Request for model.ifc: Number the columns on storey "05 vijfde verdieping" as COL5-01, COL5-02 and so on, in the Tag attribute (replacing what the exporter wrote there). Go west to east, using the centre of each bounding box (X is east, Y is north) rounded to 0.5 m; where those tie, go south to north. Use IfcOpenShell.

First a look at what the model holds.

```python
import ifcopenshell
import ifcopenshell.util.element
import ifcopenshell.util.placement

model = ifcopenshell.open("model.ifc")
print(model.schema)
storey = next(s for s in model.by_type("IfcBuildingStorey") if s.Name == "05 vijfde verdieping")
columns = [e for e in ifcopenshell.util.element.get_decomposition(storey) if e.is_a("IfcColumn")]
for e in sorted(columns, key=lambda e: e.id()):
    origin = ifcopenshell.util.placement.get_local_placement(e.ObjectPlacement)[:3, 3]
    print(e.id(), e.Tag, e.Name, origin.round(2) + 0.0, sep=" | ")
```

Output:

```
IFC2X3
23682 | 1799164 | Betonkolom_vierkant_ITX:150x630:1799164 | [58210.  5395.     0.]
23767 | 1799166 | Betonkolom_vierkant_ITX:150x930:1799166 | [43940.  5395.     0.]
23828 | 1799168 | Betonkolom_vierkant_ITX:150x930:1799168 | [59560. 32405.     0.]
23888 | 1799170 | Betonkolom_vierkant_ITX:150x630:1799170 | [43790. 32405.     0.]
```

```python
import ifcopenshell
import ifcopenshell.geom
import ifcopenshell.util.element
import ifcopenshell.util.shape

model = ifcopenshell.open("model.ifc")
settings = ifcopenshell.geom.settings()
settings.set("use-world-coords", True)


def centre(element):
    shape = ifcopenshell.geom.create_shape(settings, element)
    return ifcopenshell.util.shape.get_bbox_centroid(shape.geometry)


storey = next(s for s in model.by_type("IfcBuildingStorey") if s.Name == "05 vijfde verdieping")
columns = [e for e in ifcopenshell.util.element.get_decomposition(storey) if e.is_a("IfcColumn")]

# Insertion points can sit at a corner or the storey origin, so sort by the geometry (in metres).
centres = {e: centre(e) for e in columns}
columns.sort(key=lambda e: (round(centres[e][0] / 0.5), centres[e][1]))

for i, e in enumerate(columns, start=1):
    number = f"COL5-{i:02d}"
    e.Tag = number
    print(e.id(), number)

model.write("model-out.ifc")
```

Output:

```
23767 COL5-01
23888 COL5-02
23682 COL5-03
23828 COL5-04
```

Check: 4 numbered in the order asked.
